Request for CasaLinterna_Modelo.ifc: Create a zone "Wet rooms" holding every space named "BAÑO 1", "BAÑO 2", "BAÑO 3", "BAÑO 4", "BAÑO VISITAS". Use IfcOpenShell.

First a look at what the model holds.

```python
import ifcopenshell

model = ifcopenshell.open("CasaLinterna_Modelo.ifc")
print(model.schema)
seen = {}
for space in model.by_type("IfcSpace"):
    seen[space.LongName] = seen.get(space.LongName, 0) + 1
for name, count in sorted(seen.items(), key=str):
    print(count, "x", name)
print("zones:", [z.Name for z in model.by_type("IfcZone")][:20])
```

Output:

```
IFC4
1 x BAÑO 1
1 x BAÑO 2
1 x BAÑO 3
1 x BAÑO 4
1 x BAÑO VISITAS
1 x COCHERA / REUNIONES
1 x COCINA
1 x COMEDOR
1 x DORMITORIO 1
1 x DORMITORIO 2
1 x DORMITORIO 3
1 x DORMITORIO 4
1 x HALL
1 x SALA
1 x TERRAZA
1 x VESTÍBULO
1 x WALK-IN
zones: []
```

```python
import ifcopenshell
import ifcopenshell.api.group
import ifcopenshell.api.root

model = ifcopenshell.open("CasaLinterna_Modelo.ifc")

names = {"BAÑO 1", "BAÑO 2", "BAÑO 3", "BAÑO 4", "BAÑO VISITAS"}
spaces = [s for s in model.by_type("IfcSpace") if s.LongName in names]

zone = ifcopenshell.api.root.create_entity(model, ifc_class="IfcZone", name="Wet rooms")
ifcopenshell.api.group.assign_group(model, products=spaces, group=zone)
print(len(spaces), "spaces in", zone.Name)

model.write("CasaLinterna_Modelo-out.ifc")
```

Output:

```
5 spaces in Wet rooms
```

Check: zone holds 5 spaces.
